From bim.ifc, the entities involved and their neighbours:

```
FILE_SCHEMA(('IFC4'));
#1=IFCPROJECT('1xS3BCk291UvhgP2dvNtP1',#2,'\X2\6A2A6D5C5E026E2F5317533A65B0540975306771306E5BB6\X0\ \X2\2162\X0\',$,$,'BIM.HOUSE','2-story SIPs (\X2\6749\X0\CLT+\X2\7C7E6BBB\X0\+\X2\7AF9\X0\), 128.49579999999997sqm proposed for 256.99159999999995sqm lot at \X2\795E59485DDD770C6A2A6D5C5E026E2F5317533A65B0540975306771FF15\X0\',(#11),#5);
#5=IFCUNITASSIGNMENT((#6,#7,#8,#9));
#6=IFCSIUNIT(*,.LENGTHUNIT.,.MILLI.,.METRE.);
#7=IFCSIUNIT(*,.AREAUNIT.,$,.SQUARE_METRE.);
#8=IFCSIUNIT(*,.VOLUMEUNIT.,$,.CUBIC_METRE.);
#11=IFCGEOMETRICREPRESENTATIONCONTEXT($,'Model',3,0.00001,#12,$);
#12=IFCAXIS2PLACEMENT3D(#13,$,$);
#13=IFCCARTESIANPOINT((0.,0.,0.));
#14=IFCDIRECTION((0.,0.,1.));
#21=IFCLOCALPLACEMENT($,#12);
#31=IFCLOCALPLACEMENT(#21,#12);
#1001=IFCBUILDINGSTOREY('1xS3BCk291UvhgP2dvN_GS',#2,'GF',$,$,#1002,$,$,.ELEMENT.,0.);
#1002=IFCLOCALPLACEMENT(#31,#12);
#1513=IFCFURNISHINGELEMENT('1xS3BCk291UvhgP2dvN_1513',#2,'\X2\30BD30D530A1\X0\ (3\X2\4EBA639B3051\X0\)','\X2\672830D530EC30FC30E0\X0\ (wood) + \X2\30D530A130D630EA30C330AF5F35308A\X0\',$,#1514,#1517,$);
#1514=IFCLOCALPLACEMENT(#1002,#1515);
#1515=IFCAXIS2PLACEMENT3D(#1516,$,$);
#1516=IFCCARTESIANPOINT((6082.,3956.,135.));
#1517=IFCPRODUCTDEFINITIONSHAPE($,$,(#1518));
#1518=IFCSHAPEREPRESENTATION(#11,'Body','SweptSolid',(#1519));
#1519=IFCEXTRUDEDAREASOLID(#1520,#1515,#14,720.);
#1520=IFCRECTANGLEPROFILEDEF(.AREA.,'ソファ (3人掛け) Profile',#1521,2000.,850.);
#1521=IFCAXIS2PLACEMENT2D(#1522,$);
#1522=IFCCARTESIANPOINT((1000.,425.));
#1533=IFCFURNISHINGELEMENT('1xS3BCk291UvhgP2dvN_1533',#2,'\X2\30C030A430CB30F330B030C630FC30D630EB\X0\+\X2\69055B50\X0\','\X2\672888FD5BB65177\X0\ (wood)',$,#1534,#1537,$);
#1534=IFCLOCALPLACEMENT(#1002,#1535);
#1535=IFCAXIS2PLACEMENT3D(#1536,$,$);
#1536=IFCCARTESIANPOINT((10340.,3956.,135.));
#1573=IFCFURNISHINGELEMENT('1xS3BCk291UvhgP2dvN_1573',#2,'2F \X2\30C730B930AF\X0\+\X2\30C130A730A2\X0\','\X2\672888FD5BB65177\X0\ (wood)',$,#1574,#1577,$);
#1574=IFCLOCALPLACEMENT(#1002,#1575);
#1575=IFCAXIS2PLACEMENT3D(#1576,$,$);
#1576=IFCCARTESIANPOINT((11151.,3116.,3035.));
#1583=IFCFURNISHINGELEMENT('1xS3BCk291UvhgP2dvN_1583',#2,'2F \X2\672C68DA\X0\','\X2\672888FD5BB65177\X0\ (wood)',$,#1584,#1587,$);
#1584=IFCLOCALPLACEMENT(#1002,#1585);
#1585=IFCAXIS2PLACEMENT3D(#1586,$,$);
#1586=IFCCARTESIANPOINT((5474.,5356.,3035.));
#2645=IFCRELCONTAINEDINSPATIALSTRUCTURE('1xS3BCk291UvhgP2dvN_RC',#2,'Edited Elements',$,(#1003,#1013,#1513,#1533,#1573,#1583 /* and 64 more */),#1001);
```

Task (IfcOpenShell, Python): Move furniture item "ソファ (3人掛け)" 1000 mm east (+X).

```python
import ifcopenshell
import ifcopenshell.api.geometry
import ifcopenshell.util.placement
import ifcopenshell.util.unit

model = ifcopenshell.open("bim.ifc")
unit_scale = ifcopenshell.util.unit.calculate_unit_scale(model)

item = model.by_guid("1xS3BCk291UvhgP2dvN_1513")
matrix = ifcopenshell.util.placement.get_local_placement(item.ObjectPlacement)
matrix[0, 3] += 1 / unit_scale
ifcopenshell.api.geometry.edit_object_placement(model, product=item, matrix=matrix, is_si=False)

print(ifcopenshell.util.placement.get_local_placement(item.ObjectPlacement).round(3) + 0.0)

model.write("bim-out.ifc")
```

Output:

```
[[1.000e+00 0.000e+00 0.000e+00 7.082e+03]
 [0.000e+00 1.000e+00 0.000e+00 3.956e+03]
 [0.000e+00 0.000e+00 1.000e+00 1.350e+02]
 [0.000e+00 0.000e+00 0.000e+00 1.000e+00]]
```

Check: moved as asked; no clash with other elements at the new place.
